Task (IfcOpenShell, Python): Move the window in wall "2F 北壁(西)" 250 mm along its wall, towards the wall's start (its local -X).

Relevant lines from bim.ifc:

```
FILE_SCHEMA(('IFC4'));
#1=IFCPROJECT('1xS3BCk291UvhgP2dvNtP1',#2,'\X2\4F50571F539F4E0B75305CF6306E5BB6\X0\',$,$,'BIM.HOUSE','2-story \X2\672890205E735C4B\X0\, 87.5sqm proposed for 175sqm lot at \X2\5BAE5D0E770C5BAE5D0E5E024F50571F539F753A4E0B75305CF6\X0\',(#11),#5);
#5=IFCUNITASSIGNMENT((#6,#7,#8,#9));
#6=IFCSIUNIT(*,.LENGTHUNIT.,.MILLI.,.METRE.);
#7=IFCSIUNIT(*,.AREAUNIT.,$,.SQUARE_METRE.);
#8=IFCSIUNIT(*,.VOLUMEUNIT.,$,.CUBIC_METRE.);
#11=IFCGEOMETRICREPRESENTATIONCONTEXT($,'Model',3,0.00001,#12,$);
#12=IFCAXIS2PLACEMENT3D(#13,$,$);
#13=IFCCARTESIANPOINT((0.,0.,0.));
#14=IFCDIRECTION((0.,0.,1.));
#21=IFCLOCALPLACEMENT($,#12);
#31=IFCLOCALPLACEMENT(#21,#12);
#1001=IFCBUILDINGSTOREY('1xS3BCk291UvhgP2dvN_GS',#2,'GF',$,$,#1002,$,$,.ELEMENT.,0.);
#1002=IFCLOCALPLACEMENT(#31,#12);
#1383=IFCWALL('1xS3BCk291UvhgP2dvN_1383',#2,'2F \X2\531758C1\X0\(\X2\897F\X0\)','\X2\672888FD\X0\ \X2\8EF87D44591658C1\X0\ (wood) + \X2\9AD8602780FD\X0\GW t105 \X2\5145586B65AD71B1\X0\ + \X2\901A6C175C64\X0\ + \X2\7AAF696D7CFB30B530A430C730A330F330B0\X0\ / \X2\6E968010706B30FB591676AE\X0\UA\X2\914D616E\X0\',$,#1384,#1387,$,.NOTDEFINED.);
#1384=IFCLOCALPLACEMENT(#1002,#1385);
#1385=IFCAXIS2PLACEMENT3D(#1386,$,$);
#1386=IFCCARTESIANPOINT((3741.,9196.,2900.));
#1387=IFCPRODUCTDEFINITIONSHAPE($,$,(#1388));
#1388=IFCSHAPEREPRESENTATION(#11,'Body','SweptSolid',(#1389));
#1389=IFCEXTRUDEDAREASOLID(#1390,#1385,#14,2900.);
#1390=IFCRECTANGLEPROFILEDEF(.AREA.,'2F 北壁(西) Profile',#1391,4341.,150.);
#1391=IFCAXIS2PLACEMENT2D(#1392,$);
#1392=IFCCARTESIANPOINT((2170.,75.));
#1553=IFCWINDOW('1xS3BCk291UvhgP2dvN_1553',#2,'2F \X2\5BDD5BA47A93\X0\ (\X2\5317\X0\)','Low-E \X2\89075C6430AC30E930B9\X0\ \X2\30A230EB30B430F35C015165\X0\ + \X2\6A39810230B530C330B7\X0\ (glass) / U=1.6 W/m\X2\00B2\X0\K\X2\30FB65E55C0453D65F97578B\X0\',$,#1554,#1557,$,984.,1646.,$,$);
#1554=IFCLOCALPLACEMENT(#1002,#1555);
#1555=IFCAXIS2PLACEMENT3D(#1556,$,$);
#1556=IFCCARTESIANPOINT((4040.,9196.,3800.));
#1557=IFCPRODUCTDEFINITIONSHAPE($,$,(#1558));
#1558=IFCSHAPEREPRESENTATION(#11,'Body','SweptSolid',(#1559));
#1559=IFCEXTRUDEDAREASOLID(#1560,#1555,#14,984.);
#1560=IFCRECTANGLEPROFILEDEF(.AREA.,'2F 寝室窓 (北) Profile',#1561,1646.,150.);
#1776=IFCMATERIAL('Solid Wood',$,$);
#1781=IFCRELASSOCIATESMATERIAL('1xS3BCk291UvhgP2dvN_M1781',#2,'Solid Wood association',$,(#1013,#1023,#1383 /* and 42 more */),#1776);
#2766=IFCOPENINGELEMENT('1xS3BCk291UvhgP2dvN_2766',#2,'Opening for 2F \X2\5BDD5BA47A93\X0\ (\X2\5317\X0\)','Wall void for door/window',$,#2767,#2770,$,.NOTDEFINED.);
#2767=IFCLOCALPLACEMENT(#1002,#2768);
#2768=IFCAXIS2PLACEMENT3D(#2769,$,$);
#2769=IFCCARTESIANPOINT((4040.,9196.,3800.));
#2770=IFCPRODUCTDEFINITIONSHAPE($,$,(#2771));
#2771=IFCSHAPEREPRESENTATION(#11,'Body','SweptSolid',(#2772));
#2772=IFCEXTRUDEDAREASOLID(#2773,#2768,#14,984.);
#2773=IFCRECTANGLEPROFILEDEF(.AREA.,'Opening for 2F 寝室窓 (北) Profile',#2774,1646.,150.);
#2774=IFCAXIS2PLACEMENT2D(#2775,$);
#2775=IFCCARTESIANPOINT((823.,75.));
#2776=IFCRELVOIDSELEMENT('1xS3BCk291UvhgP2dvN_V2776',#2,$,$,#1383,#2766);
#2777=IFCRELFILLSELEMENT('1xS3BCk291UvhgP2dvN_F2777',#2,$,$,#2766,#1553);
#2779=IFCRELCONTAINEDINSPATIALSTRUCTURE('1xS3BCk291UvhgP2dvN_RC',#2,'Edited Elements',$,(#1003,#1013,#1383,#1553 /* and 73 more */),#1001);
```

```python
import ifcopenshell
import ifcopenshell.api.geometry
import ifcopenshell.util.placement

model = ifcopenshell.open("bim.ifc")

window = model.by_guid("1xS3BCk291UvhgP2dvN_1553")
opening = window.FillsVoids[0].RelatingOpeningElement
wall = opening.VoidsElements[0].RelatingBuildingElement

wall_matrix = ifcopenshell.util.placement.get_local_placement(wall.ObjectPlacement)
shift = wall_matrix[:3, 0] * -250.0
before = ifcopenshell.util.placement.get_local_placement(window.ObjectPlacement)[:3, 3].copy()

# The window is not placed relative to its opening, so move both.
for product in (opening, window):
    matrix = ifcopenshell.util.placement.get_local_placement(product.ObjectPlacement)
    matrix[:3, 3] += shift
    ifcopenshell.api.geometry.edit_object_placement(model, product=product, matrix=matrix, is_si=False)

after = ifcopenshell.util.placement.get_local_placement(window.ObjectPlacement)[:3, 3]
print("window moved by", (after - before).round(3) + 0.0)

model.write("bim_v2.ifc")
```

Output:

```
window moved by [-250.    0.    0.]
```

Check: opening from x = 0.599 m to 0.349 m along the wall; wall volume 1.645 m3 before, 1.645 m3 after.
